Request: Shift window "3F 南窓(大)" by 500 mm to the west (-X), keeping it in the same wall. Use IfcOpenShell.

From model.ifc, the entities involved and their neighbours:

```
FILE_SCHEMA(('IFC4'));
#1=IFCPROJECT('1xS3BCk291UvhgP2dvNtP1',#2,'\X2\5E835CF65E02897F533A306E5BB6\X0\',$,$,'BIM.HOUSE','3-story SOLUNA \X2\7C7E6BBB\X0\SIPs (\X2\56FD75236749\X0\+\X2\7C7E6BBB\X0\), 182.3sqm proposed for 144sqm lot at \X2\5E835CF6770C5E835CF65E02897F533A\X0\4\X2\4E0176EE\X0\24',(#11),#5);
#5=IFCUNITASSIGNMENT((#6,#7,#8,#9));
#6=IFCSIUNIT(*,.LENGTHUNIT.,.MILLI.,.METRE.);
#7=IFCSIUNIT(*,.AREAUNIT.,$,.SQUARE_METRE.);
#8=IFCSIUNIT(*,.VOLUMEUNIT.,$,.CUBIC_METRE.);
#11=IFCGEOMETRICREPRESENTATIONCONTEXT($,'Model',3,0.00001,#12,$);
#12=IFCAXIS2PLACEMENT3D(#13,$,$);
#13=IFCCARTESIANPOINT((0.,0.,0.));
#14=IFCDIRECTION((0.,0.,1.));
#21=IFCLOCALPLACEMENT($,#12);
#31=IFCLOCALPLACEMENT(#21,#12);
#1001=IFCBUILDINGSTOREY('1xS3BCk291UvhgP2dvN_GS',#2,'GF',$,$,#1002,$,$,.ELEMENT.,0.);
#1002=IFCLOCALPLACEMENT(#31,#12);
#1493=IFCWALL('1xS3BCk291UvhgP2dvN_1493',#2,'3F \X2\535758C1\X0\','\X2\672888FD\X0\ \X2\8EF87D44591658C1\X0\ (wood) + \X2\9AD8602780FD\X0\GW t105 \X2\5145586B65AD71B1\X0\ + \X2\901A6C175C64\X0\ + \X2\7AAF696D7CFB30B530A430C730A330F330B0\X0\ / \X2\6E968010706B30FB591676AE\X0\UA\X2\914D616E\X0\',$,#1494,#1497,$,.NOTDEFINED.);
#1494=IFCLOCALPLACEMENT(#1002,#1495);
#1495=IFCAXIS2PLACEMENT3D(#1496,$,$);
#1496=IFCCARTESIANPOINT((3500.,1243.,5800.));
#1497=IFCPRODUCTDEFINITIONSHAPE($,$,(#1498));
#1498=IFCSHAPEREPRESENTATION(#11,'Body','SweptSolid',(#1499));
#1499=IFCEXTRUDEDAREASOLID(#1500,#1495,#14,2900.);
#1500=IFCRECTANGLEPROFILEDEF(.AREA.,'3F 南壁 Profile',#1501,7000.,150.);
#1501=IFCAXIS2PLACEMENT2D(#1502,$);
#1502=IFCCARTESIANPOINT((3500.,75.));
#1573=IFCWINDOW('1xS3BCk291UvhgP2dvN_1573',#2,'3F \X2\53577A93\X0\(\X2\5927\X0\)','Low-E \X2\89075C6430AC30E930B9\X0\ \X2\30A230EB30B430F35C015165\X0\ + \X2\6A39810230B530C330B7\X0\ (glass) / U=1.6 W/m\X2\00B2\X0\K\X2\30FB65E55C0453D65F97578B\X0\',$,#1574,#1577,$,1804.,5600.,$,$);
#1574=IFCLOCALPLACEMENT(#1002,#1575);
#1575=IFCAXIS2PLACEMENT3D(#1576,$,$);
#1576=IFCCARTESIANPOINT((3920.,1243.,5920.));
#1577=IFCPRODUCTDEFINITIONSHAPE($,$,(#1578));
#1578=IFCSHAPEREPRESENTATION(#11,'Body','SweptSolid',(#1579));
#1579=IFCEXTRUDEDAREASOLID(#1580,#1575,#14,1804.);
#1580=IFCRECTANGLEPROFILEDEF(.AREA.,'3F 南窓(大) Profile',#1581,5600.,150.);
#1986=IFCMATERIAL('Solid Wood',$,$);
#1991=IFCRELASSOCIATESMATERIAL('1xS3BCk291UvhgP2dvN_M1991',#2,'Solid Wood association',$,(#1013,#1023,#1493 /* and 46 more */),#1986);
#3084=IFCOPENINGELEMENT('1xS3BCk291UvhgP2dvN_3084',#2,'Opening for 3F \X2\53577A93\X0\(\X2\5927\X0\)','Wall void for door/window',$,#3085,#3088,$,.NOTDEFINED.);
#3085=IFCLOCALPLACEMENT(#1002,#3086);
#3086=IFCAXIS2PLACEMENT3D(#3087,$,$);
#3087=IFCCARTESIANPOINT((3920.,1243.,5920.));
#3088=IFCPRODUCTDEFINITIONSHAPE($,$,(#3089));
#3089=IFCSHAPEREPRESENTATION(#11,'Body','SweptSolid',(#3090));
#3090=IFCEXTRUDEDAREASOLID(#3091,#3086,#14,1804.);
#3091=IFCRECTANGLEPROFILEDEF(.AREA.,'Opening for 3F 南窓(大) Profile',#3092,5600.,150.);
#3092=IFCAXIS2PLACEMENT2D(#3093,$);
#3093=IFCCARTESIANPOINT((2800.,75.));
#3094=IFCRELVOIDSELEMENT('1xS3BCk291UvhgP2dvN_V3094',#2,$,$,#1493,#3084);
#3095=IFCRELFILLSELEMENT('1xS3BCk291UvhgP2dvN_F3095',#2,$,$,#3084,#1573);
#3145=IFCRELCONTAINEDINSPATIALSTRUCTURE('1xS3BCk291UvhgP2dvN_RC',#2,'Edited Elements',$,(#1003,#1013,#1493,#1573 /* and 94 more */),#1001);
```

```python
import ifcopenshell
import ifcopenshell.api.geometry
import ifcopenshell.util.placement
import ifcopenshell.util.unit

model = ifcopenshell.open("model.ifc")
unit_scale = ifcopenshell.util.unit.calculate_unit_scale(model)

window = model.by_guid("1xS3BCk291UvhgP2dvN_1573")
opening = window.FillsVoids[0].RelatingOpeningElement
wall = opening.VoidsElements[0].RelatingBuildingElement

wall_matrix = ifcopenshell.util.placement.get_local_placement(wall.ObjectPlacement)
shift = wall_matrix[:3, 0] * -0.5 / unit_scale
before = ifcopenshell.util.placement.get_local_placement(window.ObjectPlacement)[:3, 3].copy()

# The window is not placed relative to its opening, so move both.
for product in (opening, window):
    matrix = ifcopenshell.util.placement.get_local_placement(product.ObjectPlacement)
    matrix[:3, 3] += shift
    ifcopenshell.api.geometry.edit_object_placement(model, product=product, matrix=matrix, is_si=False)

after = ifcopenshell.util.placement.get_local_placement(window.ObjectPlacement)[:3, 3]
print("window moved by", (after - before).round(3) + 0.0)

model.write("model_updated.ifc")
```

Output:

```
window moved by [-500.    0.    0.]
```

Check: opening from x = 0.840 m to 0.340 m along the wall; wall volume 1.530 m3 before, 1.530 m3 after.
